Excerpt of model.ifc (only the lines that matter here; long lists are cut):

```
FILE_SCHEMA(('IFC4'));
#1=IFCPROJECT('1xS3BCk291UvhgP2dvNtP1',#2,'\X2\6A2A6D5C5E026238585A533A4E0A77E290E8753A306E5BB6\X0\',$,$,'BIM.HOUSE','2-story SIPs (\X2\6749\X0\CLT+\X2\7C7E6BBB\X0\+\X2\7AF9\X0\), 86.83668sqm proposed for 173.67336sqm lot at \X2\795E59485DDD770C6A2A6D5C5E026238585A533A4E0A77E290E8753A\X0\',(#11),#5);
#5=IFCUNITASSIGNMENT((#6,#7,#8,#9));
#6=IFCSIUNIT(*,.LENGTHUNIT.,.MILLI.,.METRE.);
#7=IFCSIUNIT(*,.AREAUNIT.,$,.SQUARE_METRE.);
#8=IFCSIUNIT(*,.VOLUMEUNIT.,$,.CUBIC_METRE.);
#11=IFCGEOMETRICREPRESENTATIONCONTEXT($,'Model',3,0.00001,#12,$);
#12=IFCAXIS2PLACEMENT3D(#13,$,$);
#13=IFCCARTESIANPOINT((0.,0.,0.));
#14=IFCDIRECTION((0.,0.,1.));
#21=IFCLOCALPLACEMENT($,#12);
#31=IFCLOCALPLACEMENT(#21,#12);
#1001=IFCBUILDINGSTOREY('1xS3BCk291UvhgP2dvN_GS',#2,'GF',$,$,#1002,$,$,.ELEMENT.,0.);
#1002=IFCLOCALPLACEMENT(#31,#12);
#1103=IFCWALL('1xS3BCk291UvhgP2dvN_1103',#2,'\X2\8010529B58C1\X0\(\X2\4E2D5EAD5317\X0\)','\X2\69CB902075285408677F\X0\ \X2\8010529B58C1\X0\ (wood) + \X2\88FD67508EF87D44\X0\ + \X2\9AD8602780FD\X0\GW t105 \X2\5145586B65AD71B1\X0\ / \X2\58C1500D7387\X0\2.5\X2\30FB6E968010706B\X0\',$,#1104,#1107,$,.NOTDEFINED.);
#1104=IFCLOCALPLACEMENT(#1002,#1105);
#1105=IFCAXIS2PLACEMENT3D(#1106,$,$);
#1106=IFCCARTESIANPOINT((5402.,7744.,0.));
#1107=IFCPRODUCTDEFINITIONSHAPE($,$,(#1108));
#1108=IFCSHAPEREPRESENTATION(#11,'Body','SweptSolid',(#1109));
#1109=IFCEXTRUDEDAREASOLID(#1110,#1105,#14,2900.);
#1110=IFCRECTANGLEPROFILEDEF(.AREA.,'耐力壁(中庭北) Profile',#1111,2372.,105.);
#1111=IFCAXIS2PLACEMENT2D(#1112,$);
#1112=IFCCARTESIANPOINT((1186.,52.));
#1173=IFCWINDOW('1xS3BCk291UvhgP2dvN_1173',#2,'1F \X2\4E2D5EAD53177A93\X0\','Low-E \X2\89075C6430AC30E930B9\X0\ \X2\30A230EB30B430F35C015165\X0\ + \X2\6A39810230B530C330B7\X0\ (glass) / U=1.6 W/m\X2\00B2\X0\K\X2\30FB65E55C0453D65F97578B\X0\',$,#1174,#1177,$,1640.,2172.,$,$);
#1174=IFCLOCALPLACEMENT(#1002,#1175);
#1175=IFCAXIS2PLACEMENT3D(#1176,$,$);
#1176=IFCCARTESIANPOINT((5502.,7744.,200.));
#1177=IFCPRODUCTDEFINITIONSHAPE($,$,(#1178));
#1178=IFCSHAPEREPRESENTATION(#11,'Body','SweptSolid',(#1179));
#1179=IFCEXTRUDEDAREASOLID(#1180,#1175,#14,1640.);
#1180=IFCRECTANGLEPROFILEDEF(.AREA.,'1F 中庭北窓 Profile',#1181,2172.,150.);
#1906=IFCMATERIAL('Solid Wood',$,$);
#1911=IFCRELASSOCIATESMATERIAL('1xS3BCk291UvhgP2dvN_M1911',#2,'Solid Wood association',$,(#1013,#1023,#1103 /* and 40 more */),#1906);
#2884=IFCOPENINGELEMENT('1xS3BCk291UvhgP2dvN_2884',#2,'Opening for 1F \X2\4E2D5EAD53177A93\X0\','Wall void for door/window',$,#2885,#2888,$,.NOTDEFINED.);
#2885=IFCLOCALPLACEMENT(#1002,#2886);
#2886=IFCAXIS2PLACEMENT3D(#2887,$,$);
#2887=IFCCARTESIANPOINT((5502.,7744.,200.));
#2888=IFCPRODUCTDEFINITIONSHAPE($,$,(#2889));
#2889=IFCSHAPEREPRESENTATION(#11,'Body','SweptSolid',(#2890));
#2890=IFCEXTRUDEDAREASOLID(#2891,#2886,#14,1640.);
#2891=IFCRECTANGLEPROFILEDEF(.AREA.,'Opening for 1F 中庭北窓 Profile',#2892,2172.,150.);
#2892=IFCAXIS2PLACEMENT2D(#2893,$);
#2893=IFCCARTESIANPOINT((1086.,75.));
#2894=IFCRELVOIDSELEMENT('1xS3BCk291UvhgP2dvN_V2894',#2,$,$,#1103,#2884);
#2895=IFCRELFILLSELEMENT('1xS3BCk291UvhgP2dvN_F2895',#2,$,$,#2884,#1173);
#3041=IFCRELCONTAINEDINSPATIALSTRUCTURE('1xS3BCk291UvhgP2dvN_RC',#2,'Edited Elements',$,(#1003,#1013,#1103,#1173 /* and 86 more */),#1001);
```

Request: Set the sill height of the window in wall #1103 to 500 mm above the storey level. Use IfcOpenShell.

```python
import numpy as np
import ifcopenshell
import ifcopenshell.api.geometry
import ifcopenshell.geom
import ifcopenshell.util.element
import ifcopenshell.util.placement
import ifcopenshell.util.shape
import ifcopenshell.util.unit

model = ifcopenshell.open("model.ifc")
unit_scale = ifcopenshell.util.unit.calculate_unit_scale(model)

window = model.by_guid("1xS3BCk291UvhgP2dvN_1173")
opening = window.FillsVoids[0].RelatingOpeningElement
storey = ifcopenshell.util.element.get_container(window, ifc_class="IfcBuildingStorey")
level = ifcopenshell.util.placement.get_local_placement(storey.ObjectPlacement)[2, 3]

# The opening's origin need not be at the sill, so measure its lowest point.
shape = ifcopenshell.geom.create_shape(ifcopenshell.geom.settings(), opening)
bottom = ifcopenshell.util.shape.get_shape_bottom_elevation(shape, shape.geometry) / unit_scale
dz = level + 500.0 - bottom

shift = np.array([0.0, 0.0, dz])
# The window is not placed relative to its opening, so move both.
for product in (opening, window):
    matrix = ifcopenshell.util.placement.get_local_placement(product.ObjectPlacement)
    matrix[:3, 3] += shift
    ifcopenshell.api.geometry.edit_object_placement(model, product=product, matrix=matrix, is_si=False)

print(f"moved by {dz * unit_scale:+.3f} m")

model.write("model-out.ifc")
```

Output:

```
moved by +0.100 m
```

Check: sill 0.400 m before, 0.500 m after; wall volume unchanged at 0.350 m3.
